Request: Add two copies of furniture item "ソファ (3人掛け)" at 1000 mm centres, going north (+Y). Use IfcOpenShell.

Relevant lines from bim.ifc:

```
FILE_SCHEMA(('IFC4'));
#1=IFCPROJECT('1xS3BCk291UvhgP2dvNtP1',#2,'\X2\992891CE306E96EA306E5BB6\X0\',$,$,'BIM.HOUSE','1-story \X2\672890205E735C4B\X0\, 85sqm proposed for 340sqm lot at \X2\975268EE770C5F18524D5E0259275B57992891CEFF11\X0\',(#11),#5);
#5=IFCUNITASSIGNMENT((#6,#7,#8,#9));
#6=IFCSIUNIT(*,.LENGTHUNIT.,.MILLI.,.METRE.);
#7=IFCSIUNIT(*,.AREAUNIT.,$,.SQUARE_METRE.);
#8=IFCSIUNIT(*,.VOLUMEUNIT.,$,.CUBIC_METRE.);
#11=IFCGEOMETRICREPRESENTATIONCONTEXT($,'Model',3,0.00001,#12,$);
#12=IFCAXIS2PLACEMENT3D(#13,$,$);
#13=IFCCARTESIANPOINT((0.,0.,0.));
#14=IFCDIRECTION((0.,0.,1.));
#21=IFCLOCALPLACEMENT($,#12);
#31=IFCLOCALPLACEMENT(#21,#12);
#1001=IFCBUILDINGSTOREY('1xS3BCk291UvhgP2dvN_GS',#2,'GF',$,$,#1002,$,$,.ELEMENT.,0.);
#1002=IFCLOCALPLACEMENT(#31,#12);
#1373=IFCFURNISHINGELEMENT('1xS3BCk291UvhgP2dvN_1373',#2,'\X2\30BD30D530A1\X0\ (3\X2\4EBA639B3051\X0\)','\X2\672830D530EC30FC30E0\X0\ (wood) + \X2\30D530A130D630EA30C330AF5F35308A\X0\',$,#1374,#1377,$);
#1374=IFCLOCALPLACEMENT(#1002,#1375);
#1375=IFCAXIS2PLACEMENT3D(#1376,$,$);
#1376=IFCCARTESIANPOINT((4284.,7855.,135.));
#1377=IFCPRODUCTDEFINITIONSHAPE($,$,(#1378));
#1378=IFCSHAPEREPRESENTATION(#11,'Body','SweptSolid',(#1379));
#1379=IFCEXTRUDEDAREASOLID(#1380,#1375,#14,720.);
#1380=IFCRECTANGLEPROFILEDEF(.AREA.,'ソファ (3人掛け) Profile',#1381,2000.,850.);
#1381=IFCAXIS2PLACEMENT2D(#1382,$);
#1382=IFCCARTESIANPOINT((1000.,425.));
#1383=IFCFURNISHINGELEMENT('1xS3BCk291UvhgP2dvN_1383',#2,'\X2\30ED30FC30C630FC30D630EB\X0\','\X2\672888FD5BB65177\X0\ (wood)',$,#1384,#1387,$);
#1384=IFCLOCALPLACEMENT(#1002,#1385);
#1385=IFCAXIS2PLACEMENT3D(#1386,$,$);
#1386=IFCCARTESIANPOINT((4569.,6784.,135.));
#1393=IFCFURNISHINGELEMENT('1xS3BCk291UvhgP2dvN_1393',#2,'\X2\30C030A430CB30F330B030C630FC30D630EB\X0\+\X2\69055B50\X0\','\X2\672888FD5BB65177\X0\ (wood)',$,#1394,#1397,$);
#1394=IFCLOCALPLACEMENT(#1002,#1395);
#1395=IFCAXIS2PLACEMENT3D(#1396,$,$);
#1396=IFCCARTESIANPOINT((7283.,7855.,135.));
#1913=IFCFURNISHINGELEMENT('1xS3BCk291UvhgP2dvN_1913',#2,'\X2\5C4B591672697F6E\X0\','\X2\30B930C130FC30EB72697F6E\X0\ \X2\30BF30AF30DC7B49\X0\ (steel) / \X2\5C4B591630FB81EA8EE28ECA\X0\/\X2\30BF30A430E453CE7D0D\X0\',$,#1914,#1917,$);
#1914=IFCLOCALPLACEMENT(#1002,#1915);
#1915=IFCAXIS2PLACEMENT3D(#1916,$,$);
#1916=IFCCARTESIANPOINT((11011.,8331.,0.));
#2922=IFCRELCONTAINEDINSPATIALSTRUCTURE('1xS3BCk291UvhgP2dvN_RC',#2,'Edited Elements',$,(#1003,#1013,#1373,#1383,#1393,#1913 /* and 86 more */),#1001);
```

```python
import numpy as np
import ifcopenshell
import ifcopenshell.api.geometry
import ifcopenshell.api.root
import ifcopenshell.util.element
import ifcopenshell.util.placement
import ifcopenshell.util.unit

model = ifcopenshell.open("bim.ifc")
unit_scale = ifcopenshell.util.unit.calculate_unit_scale(model)


def reuse_history(source, copy):
    """copy_class also copies each property set's owner history, people and application; keep the originals."""
    for rel in copy.IsDefinedBy:
        if rel.is_a("IfcRelDefinesByProperties") and (history := rel.RelatingPropertyDefinition.OwnerHistory):
            rel.RelatingPropertyDefinition.OwnerHistory = source.OwnerHistory
            ifcopenshell.util.element.remove_deep2(model, history)


source = model.by_guid("1xS3BCk291UvhgP2dvN_1373")
base = ifcopenshell.util.placement.get_local_placement(source.ObjectPlacement)
step = np.array([0.0, 1.0, 0.0]) * 1 / unit_scale

for i in range(1, 3):
    copy = ifcopenshell.api.root.copy_class(model, product=source)
    copy.Representation = ifcopenshell.util.element.copy_deep(
        model, source.Representation, exclude=["IfcGeometricRepresentationContext", "IfcRepresentationMap"]
    )
    reuse_history(source, copy)
    matrix = base.copy()
    matrix[:3, 3] += i * step
    print("added at", matrix[:3, 3].round(3) + 0.0)
    ifcopenshell.api.geometry.edit_object_placement(model, product=copy, matrix=matrix, is_si=False)

model.write("bim_rev.ifc")
```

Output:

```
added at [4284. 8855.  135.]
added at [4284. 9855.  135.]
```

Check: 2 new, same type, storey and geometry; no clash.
